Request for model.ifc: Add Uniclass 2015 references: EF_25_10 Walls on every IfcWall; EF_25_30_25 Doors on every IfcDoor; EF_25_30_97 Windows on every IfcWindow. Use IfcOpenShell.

First a look at what the model holds.

```python
import ifcopenshell

model = ifcopenshell.open("model.ifc")
print(model.schema)
print("classifications:", [c.Name for c in model.by_type("IfcClassification")])
for ifc_class in ("IfcDoor", "IfcRoof", "IfcStair", "IfcWall", "IfcWindow"):
    print(ifc_class, len(model.by_type(ifc_class)))
```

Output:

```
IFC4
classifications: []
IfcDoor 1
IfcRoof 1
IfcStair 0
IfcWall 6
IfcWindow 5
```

```python
import ifcopenshell
import ifcopenshell.api.classification

model = ifcopenshell.open("model.ifc")

system = ifcopenshell.api.classification.add_classification(model, classification="Uniclass 2015")

codes = {
    "IfcWall": ("EF_25_10", "Walls"),
    "IfcDoor": ("EF_25_30_25", "Doors"),
    "IfcWindow": ("EF_25_30_97", "Windows"),
}
for ifc_class, (code, name) in codes.items():
    products = model.by_type(ifc_class)
    ifcopenshell.api.classification.add_reference(
        model, products=products, classification=system, identification=code, name=name
    )
    print(code, len(products))

model.write("model_v2.ifc")
```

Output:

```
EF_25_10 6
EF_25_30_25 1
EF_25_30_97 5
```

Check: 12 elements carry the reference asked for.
